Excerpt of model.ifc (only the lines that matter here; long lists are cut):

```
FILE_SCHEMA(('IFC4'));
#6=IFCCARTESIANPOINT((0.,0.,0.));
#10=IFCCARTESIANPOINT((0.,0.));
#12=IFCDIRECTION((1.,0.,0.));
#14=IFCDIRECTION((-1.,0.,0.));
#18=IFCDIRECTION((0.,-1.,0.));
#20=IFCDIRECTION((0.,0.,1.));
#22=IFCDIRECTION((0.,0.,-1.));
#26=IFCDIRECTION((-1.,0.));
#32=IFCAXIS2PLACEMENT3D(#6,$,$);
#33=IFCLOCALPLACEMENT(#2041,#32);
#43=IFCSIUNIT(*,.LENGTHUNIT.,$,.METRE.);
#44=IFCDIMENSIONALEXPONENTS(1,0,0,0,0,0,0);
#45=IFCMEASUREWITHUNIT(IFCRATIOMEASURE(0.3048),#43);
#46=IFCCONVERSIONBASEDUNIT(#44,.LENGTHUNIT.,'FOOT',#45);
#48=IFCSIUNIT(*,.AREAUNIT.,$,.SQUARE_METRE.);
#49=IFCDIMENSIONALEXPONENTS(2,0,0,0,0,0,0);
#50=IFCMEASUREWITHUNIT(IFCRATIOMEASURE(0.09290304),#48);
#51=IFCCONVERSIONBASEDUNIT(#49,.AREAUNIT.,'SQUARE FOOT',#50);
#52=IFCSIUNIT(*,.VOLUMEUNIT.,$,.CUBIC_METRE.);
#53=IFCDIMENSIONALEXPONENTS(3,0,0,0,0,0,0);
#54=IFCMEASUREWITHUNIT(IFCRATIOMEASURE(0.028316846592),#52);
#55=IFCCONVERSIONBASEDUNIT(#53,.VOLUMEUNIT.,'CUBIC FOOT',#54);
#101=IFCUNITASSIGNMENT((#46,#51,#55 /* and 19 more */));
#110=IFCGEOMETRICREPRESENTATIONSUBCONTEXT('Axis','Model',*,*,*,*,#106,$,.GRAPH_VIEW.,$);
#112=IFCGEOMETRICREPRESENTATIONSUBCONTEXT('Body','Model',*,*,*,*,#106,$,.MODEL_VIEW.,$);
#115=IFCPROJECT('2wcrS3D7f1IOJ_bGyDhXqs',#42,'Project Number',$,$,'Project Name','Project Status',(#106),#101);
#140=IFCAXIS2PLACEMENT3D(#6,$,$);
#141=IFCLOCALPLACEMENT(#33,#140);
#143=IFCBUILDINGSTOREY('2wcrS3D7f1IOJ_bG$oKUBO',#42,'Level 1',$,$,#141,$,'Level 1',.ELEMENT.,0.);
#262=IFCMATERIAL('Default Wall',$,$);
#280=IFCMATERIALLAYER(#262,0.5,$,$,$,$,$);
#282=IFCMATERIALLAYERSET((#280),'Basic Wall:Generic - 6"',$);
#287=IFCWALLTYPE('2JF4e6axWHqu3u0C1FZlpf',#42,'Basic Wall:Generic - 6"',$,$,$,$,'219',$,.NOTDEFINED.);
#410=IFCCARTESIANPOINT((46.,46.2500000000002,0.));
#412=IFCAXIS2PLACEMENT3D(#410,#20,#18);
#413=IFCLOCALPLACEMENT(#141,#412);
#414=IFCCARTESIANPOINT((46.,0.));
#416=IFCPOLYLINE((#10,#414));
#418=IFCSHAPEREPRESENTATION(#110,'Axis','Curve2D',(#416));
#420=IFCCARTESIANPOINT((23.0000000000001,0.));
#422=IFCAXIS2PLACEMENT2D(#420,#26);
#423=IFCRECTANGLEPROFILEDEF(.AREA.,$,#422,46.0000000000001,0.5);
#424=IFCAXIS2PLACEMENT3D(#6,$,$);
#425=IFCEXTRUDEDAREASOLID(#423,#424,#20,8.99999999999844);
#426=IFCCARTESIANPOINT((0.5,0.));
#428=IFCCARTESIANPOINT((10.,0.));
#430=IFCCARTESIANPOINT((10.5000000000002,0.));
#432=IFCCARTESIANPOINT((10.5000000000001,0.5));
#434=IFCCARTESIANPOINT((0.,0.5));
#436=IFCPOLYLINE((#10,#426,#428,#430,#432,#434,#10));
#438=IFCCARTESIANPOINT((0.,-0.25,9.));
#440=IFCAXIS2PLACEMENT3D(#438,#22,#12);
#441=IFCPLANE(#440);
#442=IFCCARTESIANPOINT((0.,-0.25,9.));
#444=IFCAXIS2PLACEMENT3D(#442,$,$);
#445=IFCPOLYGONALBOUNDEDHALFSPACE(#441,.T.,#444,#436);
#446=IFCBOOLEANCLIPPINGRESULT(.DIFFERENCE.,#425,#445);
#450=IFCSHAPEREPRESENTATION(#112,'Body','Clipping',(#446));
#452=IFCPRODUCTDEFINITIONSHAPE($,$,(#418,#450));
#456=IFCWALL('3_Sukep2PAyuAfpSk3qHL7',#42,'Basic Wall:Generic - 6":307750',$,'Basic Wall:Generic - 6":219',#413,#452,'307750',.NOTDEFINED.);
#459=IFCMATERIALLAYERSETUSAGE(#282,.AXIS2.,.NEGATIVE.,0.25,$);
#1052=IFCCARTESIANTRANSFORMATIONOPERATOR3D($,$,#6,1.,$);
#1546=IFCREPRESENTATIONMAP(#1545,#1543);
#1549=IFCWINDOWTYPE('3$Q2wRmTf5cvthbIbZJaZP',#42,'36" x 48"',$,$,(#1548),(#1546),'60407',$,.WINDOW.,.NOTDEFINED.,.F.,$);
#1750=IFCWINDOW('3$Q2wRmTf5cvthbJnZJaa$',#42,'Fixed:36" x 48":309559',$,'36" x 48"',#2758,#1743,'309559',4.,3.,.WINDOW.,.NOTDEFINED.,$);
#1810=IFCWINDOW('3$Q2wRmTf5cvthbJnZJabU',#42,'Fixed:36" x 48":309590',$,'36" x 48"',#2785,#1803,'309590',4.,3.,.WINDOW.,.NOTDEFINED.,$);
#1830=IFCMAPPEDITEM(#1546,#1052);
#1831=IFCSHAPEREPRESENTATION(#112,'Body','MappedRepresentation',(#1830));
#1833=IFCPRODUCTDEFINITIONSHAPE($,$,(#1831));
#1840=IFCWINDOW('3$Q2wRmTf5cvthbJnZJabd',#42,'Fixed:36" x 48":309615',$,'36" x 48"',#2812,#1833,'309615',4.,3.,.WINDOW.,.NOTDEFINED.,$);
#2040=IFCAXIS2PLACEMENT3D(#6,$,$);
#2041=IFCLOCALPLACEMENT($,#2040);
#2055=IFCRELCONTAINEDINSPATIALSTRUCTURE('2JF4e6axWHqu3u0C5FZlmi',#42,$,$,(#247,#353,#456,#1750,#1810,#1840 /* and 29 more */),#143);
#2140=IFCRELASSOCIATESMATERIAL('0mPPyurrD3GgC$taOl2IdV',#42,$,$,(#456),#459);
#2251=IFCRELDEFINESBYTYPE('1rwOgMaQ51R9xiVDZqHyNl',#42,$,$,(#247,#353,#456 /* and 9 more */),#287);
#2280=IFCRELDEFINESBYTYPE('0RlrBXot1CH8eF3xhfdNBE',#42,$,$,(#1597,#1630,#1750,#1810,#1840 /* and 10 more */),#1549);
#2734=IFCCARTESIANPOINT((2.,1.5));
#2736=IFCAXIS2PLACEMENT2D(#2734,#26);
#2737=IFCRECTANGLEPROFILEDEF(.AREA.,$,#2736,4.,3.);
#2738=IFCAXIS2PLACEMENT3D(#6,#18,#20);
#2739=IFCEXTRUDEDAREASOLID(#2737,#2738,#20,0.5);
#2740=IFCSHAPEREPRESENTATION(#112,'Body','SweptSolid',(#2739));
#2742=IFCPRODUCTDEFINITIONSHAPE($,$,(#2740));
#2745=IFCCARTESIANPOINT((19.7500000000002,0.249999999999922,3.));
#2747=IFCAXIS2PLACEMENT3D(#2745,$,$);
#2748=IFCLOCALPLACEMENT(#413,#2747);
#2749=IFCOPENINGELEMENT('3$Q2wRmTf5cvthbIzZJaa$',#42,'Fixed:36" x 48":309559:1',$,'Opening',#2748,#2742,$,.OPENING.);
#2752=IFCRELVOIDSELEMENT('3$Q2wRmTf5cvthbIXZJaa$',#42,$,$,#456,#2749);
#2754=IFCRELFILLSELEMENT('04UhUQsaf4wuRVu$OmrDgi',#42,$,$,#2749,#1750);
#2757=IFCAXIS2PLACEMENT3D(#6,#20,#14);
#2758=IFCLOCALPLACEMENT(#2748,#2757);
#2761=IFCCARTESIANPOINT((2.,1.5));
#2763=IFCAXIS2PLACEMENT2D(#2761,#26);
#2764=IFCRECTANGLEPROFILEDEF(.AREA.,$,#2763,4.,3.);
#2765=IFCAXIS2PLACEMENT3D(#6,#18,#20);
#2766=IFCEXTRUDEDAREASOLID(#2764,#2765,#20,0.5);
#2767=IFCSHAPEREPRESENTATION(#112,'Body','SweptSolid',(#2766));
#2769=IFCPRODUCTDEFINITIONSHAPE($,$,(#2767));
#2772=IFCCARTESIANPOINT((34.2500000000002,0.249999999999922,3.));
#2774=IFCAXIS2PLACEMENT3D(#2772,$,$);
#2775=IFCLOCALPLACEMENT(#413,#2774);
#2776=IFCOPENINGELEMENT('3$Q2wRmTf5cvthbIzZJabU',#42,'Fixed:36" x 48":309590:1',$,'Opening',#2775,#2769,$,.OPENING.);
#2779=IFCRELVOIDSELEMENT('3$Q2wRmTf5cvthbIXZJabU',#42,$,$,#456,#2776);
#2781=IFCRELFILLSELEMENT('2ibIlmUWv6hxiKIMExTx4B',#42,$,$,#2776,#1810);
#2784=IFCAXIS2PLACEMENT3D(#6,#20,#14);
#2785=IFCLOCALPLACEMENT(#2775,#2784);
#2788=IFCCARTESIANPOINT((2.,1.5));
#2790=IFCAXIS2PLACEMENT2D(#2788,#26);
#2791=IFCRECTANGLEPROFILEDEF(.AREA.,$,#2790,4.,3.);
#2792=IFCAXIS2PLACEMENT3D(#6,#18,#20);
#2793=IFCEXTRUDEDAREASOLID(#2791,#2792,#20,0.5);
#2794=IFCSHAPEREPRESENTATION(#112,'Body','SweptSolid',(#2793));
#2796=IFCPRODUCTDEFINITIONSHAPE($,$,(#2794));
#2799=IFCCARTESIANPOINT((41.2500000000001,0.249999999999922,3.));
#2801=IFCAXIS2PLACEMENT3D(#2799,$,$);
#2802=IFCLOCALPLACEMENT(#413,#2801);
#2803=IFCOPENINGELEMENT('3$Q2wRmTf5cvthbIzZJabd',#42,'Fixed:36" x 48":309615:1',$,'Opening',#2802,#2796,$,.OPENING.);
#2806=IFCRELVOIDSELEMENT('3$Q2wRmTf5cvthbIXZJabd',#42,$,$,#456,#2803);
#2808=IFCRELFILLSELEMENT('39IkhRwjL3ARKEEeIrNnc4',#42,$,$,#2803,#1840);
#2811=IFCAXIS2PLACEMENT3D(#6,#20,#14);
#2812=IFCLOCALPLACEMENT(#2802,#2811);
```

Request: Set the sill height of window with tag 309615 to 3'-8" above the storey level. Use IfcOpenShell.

```python
import numpy as np
import ifcopenshell
import ifcopenshell.api.geometry
import ifcopenshell.geom
import ifcopenshell.util.element
import ifcopenshell.util.placement
import ifcopenshell.util.shape
import ifcopenshell.util.unit

model = ifcopenshell.open("model.ifc")
unit_scale = ifcopenshell.util.unit.calculate_unit_scale(model)

window = model.by_guid("3$Q2wRmTf5cvthbJnZJabd")
opening = window.FillsVoids[0].RelatingOpeningElement
storey = ifcopenshell.util.element.get_container(window, ifc_class="IfcBuildingStorey")
level = ifcopenshell.util.placement.get_local_placement(storey.ObjectPlacement)[2, 3]

# The opening's origin need not be at the sill, so measure its lowest point.
shape = ifcopenshell.geom.create_shape(ifcopenshell.geom.settings(), opening)
bottom = ifcopenshell.util.shape.get_shape_bottom_elevation(shape, shape.geometry) / unit_scale
dz = level + 44 * 0.0254 / unit_scale - bottom

shift = np.array([0.0, 0.0, dz])
# The window is placed relative to its opening, so it follows when the opening moves.
matrix = ifcopenshell.util.placement.get_local_placement(opening.ObjectPlacement)
matrix[:3, 3] += shift
ifcopenshell.api.geometry.edit_object_placement(
    model, product=opening, matrix=matrix, is_si=False, should_transform_children=True
)

print(f"moved by {dz * unit_scale:+.3f} m")

model.write("model-out.ifc")
```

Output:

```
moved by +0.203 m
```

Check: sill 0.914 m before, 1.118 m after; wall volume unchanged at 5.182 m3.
